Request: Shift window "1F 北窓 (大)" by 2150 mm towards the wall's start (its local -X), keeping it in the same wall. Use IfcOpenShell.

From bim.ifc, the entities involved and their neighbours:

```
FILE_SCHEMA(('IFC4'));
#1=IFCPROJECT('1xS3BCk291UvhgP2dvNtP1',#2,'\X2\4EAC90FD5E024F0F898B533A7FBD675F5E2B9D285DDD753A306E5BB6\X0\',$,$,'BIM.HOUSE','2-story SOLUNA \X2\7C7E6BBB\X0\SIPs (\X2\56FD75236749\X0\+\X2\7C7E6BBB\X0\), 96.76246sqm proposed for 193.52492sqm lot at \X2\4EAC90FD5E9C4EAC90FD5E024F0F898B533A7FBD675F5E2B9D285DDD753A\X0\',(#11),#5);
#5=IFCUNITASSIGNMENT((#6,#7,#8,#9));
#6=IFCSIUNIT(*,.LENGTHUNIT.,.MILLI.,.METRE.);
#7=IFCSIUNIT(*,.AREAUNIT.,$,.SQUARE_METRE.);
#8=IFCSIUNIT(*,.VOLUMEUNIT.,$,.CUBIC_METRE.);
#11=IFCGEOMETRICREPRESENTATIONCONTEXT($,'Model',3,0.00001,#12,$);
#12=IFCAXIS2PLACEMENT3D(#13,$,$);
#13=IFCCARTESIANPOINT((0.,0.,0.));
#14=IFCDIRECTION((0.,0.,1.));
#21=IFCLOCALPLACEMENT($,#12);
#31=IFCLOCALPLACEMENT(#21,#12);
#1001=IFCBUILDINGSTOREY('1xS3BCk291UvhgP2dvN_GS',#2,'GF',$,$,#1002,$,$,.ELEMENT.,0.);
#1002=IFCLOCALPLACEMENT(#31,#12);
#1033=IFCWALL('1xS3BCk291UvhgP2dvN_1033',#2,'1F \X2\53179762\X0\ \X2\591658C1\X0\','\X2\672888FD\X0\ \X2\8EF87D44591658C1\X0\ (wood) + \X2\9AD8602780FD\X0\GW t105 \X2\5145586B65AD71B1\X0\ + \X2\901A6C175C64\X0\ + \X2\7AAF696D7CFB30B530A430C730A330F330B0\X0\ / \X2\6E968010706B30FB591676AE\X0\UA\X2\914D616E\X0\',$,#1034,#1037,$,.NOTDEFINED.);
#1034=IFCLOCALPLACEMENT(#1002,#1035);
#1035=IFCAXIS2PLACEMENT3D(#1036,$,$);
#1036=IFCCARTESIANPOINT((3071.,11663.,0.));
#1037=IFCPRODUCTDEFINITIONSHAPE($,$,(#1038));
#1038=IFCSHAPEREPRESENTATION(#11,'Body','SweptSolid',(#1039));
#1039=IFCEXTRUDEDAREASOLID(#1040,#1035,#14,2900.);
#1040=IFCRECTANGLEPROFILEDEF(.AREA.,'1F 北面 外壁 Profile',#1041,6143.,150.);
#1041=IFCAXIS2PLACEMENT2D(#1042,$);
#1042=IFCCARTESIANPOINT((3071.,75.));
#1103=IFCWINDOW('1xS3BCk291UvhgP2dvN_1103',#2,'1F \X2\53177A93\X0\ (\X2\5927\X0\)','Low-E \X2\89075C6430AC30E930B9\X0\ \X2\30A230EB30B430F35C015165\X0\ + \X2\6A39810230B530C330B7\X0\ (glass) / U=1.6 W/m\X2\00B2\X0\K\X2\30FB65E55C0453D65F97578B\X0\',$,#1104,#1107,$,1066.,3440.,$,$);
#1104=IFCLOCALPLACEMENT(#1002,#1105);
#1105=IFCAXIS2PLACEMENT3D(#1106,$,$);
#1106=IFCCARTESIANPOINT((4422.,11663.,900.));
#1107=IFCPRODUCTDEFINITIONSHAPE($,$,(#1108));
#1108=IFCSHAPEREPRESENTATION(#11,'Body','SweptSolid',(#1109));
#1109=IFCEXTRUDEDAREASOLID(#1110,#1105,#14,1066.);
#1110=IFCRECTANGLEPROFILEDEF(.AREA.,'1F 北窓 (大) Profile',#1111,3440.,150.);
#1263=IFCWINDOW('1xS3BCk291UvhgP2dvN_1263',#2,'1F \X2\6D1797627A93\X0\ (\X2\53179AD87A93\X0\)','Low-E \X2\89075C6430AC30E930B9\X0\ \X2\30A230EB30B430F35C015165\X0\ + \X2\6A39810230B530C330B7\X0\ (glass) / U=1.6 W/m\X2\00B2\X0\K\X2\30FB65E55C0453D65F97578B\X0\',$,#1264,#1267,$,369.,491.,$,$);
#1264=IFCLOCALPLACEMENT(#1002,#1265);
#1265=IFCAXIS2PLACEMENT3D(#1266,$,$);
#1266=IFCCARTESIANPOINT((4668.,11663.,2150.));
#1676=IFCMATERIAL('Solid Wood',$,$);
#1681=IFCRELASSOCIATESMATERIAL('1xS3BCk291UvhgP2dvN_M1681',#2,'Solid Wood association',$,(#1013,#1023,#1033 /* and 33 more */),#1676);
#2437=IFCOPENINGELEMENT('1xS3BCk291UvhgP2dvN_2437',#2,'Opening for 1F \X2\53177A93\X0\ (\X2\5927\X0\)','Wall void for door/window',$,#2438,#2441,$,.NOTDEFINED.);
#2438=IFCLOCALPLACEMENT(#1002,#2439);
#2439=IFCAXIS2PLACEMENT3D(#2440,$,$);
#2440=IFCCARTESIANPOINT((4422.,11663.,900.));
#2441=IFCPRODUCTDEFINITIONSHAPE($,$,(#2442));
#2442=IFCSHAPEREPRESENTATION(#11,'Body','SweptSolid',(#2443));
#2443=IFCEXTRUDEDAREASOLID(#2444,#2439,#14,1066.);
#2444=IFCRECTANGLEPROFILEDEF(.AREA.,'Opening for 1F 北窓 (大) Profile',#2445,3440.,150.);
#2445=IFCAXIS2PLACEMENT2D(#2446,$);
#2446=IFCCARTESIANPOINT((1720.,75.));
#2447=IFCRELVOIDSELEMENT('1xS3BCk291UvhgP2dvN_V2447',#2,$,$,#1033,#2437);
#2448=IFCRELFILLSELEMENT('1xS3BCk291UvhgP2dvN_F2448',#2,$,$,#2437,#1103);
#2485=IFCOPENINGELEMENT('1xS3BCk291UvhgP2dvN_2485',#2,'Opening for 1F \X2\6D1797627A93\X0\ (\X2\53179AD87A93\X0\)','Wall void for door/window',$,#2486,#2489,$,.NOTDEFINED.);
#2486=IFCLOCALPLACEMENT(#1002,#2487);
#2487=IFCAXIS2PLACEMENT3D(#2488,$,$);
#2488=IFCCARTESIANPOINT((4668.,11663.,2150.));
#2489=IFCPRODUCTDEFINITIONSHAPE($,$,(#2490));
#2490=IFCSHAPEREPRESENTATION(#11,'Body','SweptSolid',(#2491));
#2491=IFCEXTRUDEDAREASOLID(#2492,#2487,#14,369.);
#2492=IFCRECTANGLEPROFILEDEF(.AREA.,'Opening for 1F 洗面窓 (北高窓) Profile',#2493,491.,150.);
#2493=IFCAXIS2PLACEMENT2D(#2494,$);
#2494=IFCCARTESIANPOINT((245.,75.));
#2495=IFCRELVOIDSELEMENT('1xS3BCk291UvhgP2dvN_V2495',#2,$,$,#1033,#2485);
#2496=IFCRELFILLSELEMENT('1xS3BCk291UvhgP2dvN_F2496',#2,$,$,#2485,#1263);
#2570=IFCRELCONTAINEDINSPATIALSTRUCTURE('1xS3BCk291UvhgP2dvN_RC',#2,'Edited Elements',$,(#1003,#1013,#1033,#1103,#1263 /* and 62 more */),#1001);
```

```python
import ifcopenshell
import ifcopenshell.api.geometry
import ifcopenshell.util.placement
import ifcopenshell.util.unit

model = ifcopenshell.open("bim.ifc")
unit_scale = ifcopenshell.util.unit.calculate_unit_scale(model)

window = model.by_guid("1xS3BCk291UvhgP2dvN_1103")
opening = window.FillsVoids[0].RelatingOpeningElement
wall = opening.VoidsElements[0].RelatingBuildingElement

wall_matrix = ifcopenshell.util.placement.get_local_placement(wall.ObjectPlacement)
shift = wall_matrix[:3, 0] * -2.15 / unit_scale
before = ifcopenshell.util.placement.get_local_placement(window.ObjectPlacement)[:3, 3].copy()

# The window is not placed relative to its opening, so move both.
for product in (opening, window):
    matrix = ifcopenshell.util.placement.get_local_placement(product.ObjectPlacement)
    matrix[:3, 3] += shift
    ifcopenshell.api.geometry.edit_object_placement(model, product=product, matrix=matrix, is_si=False)

after = ifcopenshell.util.placement.get_local_placement(window.ObjectPlacement)[:3, 3]
print("window moved by", (after - before).round(3) + 0.0)

model.write("bim_rev.ifc")
```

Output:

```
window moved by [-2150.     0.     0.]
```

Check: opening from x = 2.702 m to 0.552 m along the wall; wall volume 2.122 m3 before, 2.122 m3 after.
